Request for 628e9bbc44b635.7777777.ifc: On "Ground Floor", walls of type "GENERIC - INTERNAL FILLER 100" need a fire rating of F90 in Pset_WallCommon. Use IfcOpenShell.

First a look at what the model holds.

```python
import ifcopenshell
import ifcopenshell.util.element

model = ifcopenshell.open("628e9bbc44b635.7777777.ifc")
print(model.schema)
storey = next(s for s in model.by_type("IfcBuildingStorey") if s.Name == "Ground Floor")
walls = [e for e in ifcopenshell.util.element.get_decomposition(storey) if e.is_a("IfcWall")]
seen = {}
for e in walls:
    element_type = ifcopenshell.util.element.get_type(e)
    key = (element_type.Name if element_type != e and element_type else None, ifcopenshell.util.element.get_pset(e, "Pset_WallCommon", "FireRating"))
    seen[key] = seen.get(key, 0) + 1
for (name, value), count in sorted(seen.items(), key=str):
    print(count, "x", name, "|", value)
```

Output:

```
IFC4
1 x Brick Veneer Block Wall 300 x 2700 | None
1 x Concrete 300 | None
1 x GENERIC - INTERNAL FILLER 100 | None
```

```python
import ifcopenshell
import ifcopenshell.api.pset
import ifcopenshell.util.element

model = ifcopenshell.open("628e9bbc44b635.7777777.ifc")

storey = next(s for s in model.by_type("IfcBuildingStorey") if s.Name == "Ground Floor")
walls = [e for e in ifcopenshell.util.element.get_decomposition(storey) if e.is_a("IfcWall")]

count = 0
for e in walls:
    element_type = ifcopenshell.util.element.get_type(e)
    if element_type in (None, e) or element_type.Name != "GENERIC - INTERNAL FILLER 100":
        continue
    # add_pset returns the element's existing set when there is one.
    pset = ifcopenshell.api.pset.add_pset(model, product=e, name="Pset_WallCommon")
    ifcopenshell.api.pset.edit_pset(model, pset=pset, properties={"FireRating": "F90"})
    count += 1

print(count, "walls updated")

model.write("628e9bbc44b635.7777777-out.ifc")
```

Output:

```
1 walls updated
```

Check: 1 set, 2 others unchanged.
